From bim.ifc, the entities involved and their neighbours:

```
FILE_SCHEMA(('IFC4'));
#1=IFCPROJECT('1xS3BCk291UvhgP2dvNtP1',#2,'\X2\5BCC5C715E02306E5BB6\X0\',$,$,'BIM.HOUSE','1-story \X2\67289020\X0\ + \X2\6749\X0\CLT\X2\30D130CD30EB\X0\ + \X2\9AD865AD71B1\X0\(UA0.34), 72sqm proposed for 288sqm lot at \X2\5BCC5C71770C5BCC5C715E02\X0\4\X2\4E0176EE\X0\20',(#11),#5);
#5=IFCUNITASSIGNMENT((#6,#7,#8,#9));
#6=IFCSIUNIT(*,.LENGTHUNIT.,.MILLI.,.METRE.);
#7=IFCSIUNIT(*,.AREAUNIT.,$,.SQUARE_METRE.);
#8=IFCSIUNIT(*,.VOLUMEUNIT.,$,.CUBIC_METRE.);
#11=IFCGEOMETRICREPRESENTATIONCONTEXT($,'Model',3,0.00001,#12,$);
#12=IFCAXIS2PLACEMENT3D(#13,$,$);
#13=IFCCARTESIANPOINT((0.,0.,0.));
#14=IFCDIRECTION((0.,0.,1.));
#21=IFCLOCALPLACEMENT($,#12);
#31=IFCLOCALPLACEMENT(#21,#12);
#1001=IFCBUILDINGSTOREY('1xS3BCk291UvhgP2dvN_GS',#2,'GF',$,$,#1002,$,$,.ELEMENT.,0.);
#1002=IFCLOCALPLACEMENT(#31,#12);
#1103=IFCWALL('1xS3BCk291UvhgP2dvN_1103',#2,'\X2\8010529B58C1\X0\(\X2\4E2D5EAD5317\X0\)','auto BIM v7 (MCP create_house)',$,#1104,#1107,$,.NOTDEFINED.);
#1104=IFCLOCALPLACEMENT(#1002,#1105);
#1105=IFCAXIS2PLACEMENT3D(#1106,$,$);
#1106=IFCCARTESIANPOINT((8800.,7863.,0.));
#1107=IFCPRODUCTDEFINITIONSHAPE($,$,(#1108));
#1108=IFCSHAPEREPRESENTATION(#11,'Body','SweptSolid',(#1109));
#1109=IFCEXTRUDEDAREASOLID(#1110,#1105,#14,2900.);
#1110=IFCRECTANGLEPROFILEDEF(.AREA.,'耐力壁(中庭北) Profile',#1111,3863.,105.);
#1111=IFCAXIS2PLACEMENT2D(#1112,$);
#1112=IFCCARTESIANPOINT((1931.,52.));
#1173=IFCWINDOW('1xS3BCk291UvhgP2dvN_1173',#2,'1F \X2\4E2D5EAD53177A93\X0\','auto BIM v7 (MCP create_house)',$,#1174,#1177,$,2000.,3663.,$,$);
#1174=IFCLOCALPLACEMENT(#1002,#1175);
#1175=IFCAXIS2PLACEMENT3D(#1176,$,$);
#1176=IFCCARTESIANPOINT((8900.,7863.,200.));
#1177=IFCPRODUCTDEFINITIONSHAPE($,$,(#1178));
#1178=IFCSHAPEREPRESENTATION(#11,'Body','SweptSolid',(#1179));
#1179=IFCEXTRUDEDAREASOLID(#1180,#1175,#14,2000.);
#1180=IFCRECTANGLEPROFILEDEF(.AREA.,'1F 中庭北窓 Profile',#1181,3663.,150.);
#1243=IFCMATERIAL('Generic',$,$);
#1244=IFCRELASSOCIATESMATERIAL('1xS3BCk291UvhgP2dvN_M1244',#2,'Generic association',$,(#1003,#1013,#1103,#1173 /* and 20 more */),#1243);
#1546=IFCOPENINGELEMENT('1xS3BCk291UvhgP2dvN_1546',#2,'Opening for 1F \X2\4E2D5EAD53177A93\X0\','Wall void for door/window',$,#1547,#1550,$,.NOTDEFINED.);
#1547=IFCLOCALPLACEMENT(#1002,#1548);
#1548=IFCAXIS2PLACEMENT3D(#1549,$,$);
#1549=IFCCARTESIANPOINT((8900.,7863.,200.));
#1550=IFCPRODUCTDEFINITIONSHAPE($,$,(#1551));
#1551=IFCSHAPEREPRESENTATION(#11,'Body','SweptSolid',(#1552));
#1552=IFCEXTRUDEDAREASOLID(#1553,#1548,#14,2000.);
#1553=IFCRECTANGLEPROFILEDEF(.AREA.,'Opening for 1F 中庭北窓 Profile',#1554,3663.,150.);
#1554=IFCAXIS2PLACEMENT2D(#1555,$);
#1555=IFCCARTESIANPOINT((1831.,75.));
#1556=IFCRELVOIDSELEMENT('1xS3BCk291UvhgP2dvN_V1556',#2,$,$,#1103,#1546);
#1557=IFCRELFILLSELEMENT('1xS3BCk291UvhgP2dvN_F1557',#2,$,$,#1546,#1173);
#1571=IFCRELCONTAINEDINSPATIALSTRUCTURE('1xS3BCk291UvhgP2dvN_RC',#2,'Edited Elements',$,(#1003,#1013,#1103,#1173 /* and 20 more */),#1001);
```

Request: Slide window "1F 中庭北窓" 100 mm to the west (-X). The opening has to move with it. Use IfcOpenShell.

```python
import ifcopenshell
import ifcopenshell.api.geometry
import ifcopenshell.util.placement
import ifcopenshell.util.unit

model = ifcopenshell.open("bim.ifc")
unit_scale = ifcopenshell.util.unit.calculate_unit_scale(model)

window = model.by_guid("1xS3BCk291UvhgP2dvN_1173")
opening = window.FillsVoids[0].RelatingOpeningElement
wall = opening.VoidsElements[0].RelatingBuildingElement

wall_matrix = ifcopenshell.util.placement.get_local_placement(wall.ObjectPlacement)
shift = wall_matrix[:3, 0] * -0.1 / unit_scale
before = ifcopenshell.util.placement.get_local_placement(window.ObjectPlacement)[:3, 3].copy()

# The window is not placed relative to its opening, so move both.
for product in (opening, window):
    matrix = ifcopenshell.util.placement.get_local_placement(product.ObjectPlacement)
    matrix[:3, 3] += shift
    ifcopenshell.api.geometry.edit_object_placement(model, product=product, matrix=matrix, is_si=False)

after = ifcopenshell.util.placement.get_local_placement(window.ObjectPlacement)[:3, 3]
print("window moved by", (after - before).round(3) + 0.0)

model.write("bim_edited.ifc")
```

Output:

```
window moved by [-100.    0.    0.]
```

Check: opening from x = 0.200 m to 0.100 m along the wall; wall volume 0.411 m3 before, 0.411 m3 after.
